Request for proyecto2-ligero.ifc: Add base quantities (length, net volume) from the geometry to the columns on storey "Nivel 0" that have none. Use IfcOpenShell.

First a look at what the model holds.

```python
import ifcopenshell
import ifcopenshell.util.element
import ifcopenshell.util.unit

model = ifcopenshell.open("proyecto2-ligero.ifc")
print(model.schema)
for unit_type in ("LENGTHUNIT", "AREAUNIT", "VOLUMEUNIT"):
    print(unit_type, ifcopenshell.util.unit.calculate_unit_scale(model, unit_type))
storey = next(s for s in model.by_type("IfcBuildingStorey") if s.Name == "Nivel 0")
columns = [e for e in ifcopenshell.util.element.get_decomposition(storey) if e.is_a("IfcColumn")]
for e in sorted(columns, key=lambda e: e.id()):
    print(e.id(), e.is_a(), e.Name, list(ifcopenshell.util.element.get_psets(e, qtos_only=True)), sep=" | ")
```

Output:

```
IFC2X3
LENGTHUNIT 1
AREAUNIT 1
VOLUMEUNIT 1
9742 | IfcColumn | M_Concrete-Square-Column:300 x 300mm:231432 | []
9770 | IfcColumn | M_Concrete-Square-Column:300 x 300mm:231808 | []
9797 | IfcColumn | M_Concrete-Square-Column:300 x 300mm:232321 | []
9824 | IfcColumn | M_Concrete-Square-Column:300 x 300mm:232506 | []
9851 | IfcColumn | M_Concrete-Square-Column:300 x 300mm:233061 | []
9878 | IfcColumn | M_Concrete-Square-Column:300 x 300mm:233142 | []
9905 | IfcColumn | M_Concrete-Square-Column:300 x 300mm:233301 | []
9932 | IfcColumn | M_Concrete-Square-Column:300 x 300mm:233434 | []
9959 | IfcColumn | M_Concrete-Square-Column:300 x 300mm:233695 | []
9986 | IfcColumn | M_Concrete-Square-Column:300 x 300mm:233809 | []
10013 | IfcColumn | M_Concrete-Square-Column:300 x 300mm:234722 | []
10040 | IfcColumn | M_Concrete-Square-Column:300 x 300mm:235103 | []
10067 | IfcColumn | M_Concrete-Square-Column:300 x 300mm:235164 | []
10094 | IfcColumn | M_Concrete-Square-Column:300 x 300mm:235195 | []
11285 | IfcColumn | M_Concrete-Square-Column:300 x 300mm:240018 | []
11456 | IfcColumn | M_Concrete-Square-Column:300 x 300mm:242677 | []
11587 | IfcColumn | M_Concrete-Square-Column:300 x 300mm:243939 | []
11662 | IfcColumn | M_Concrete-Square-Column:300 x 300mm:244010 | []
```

```python
import ifcopenshell
import ifcopenshell.api.pset
import ifcopenshell.geom
import ifcopenshell.util.element
import ifcopenshell.util.shape
import ifcopenshell.util.unit

model = ifcopenshell.open("proyecto2-ligero.ifc")
unit_scale = ifcopenshell.util.unit.calculate_unit_scale(model)
volume_scale = ifcopenshell.util.unit.calculate_unit_scale(model, "VOLUMEUNIT")
settings = ifcopenshell.geom.settings()

storey = next(s for s in model.by_type("IfcBuildingStorey") if s.Name == "Nivel 0")
columns = [e for e in ifcopenshell.util.element.get_decomposition(storey) if e.is_a("IfcColumn")]

for e in sorted(columns, key=lambda e: e.id()):
    if ifcopenshell.util.element.get_psets(e, qtos_only=True, should_inherit=False):
        continue
    # Geometry comes back in metres, in the element's own axes.
    shape = ifcopenshell.geom.create_shape(settings, e)
    values = {
        "Length": ifcopenshell.util.shape.get_z(shape.geometry) / unit_scale,
        "NetVolume": ifcopenshell.util.shape.get_volume(shape.geometry) / volume_scale,
    }
    qto = ifcopenshell.api.pset.add_qto(model, product=e, name="BaseQuantities")
    ifcopenshell.api.pset.edit_qto(model, qto=qto, properties=values)
    print(e.id(), {k: round(v, 3) for k, v in values.items()})

model.write("proyecto2-ligero_v2.ifc")
```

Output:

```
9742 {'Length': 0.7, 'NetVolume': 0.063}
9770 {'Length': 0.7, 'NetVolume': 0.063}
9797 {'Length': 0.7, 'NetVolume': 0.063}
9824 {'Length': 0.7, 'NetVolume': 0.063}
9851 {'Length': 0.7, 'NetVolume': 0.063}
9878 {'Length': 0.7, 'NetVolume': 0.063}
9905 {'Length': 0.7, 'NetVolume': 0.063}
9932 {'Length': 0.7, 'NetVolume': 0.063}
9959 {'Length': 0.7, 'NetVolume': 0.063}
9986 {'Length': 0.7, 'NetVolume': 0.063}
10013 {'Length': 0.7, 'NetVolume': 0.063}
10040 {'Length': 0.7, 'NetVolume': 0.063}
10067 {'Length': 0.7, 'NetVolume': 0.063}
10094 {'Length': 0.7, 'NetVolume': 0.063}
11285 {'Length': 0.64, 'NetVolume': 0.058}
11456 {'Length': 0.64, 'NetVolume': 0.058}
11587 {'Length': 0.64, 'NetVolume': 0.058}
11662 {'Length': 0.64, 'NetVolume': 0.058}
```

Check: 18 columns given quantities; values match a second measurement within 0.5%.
